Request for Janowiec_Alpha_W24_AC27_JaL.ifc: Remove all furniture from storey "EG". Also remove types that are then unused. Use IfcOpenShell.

First a look at what the model holds.

```python
import ifcopenshell
import ifcopenshell.util.element

model = ifcopenshell.open("Janowiec_Alpha_W24_AC27_JaL.ifc")
print(model.schema)
storey = next(s for s in model.by_type("IfcBuildingStorey") if s.Name == "EG")
furniture = [e for e in ifcopenshell.util.element.get_decomposition(storey) if e.is_a("IfcFurnishingElement")]
seen = {}
for e in furniture:
    element_type = ifcopenshell.util.element.get_type(e)
    name = element_type.Name if element_type not in (None, e) else None
    seen[name] = seen.get(name, 0) + 1
for name, count in sorted(seen.items(), key=str):
    print(count, "x", name)
```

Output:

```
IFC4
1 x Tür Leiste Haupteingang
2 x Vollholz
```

```python
import ifcopenshell
import ifcopenshell.api.root
import ifcopenshell.util.element

model = ifcopenshell.open("Janowiec_Alpha_W24_AC27_JaL.ifc")

storey = next(s for s in model.by_type("IfcBuildingStorey") if s.Name == "EG")
furniture = [e for e in ifcopenshell.util.element.get_decomposition(storey) if e.is_a("IfcFurnishingElement")]
types = {ifcopenshell.util.element.get_type(e) for e in furniture} - {None, *furniture}

for e in furniture:
    ifcopenshell.api.root.remove_product(model, product=e)
print(len(furniture), "removed")

unused = [t for t in types if not ifcopenshell.util.element.get_types(t)]
for t in unused:
    ifcopenshell.api.root.remove_product(model, product=t)
print(len(unused), "unused types removed")

model.write("Janowiec_Alpha_W24_AC27_JaL_v2.ifc")
```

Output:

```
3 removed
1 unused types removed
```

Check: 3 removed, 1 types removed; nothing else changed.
